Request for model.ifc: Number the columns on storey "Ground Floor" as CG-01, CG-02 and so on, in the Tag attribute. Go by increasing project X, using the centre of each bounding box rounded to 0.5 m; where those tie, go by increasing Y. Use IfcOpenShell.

First a look at what the model holds.

```python
import ifcopenshell
import ifcopenshell.util.element
import ifcopenshell.util.placement

model = ifcopenshell.open("model.ifc")
print(model.schema)
storey = next(s for s in model.by_type("IfcBuildingStorey") if s.Name == "Ground Floor")
columns = [e for e in ifcopenshell.util.element.get_decomposition(storey) if e.is_a("IfcColumn")]
for e in sorted(columns, key=lambda e: e.id()):
    origin = ifcopenshell.util.placement.get_local_placement(e.ObjectPlacement)[:3, 3]
    print(e.id(), e.Tag, e.Name, origin.round(2) + 0.0, sep=" | ")
```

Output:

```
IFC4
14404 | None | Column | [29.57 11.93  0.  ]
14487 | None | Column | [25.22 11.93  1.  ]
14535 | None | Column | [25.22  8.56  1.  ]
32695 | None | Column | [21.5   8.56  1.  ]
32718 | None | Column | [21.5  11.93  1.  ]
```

```python
import ifcopenshell
import ifcopenshell.geom
import ifcopenshell.util.element
import ifcopenshell.util.shape

model = ifcopenshell.open("model.ifc")
settings = ifcopenshell.geom.settings()
settings.set("use-world-coords", True)


def centre(element):
    shape = ifcopenshell.geom.create_shape(settings, element)
    return ifcopenshell.util.shape.get_bbox_centroid(shape.geometry)


storey = next(s for s in model.by_type("IfcBuildingStorey") if s.Name == "Ground Floor")
columns = [e for e in ifcopenshell.util.element.get_decomposition(storey) if e.is_a("IfcColumn")]

# Insertion points can sit at a corner or the storey origin, so sort by the geometry (in metres).
centres = {e: centre(e) for e in columns}
columns.sort(key=lambda e: (round(centres[e][0] / 0.5), centres[e][1]))

for i, e in enumerate(columns, start=1):
    number = f"CG-{i:02d}"
    e.Tag = number
    print(e.id(), number)

model.write("model_v2.ifc")
```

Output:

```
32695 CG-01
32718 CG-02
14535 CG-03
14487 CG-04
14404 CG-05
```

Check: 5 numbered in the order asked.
